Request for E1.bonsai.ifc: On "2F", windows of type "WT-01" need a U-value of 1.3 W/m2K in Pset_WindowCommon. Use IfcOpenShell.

First a look at what the model holds.

```python
import ifcopenshell
import ifcopenshell.util.element

model = ifcopenshell.open("E1.bonsai.ifc")
print(model.schema)
storey = next(s for s in model.by_type("IfcBuildingStorey") if s.Name == "2F")
windows = [e for e in ifcopenshell.util.element.get_decomposition(storey) if e.is_a("IfcWindow")]
seen = {}
for e in windows:
    element_type = ifcopenshell.util.element.get_type(e)
    key = (element_type.Name if element_type != e and element_type else None, ifcopenshell.util.element.get_pset(e, "Pset_WindowCommon", "ThermalTransmittance"))
    seen[key] = seen.get(key, 0) + 1
for (name, value), count in sorted(seen.items(), key=str):
    print(count, "x", name, "|", value)
```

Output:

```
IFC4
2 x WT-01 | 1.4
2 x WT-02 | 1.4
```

```python
import ifcopenshell
import ifcopenshell.api.pset
import ifcopenshell.util.element

model = ifcopenshell.open("E1.bonsai.ifc")

storey = next(s for s in model.by_type("IfcBuildingStorey") if s.Name == "2F")
windows = [e for e in ifcopenshell.util.element.get_decomposition(storey) if e.is_a("IfcWindow")]

count = 0
for e in windows:
    element_type = ifcopenshell.util.element.get_type(e)
    if element_type in (None, e) or element_type.Name != "WT-01":
        continue
    # add_pset returns the element's existing set when there is one.
    pset = ifcopenshell.api.pset.add_pset(model, product=e, name="Pset_WindowCommon")
    ifcopenshell.api.pset.edit_pset(model, pset=pset, properties={"ThermalTransmittance": 1.3})
    count += 1

print(count, "windows updated")

model.write("E1.bonsai-out.ifc")
```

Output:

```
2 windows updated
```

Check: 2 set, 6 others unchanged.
